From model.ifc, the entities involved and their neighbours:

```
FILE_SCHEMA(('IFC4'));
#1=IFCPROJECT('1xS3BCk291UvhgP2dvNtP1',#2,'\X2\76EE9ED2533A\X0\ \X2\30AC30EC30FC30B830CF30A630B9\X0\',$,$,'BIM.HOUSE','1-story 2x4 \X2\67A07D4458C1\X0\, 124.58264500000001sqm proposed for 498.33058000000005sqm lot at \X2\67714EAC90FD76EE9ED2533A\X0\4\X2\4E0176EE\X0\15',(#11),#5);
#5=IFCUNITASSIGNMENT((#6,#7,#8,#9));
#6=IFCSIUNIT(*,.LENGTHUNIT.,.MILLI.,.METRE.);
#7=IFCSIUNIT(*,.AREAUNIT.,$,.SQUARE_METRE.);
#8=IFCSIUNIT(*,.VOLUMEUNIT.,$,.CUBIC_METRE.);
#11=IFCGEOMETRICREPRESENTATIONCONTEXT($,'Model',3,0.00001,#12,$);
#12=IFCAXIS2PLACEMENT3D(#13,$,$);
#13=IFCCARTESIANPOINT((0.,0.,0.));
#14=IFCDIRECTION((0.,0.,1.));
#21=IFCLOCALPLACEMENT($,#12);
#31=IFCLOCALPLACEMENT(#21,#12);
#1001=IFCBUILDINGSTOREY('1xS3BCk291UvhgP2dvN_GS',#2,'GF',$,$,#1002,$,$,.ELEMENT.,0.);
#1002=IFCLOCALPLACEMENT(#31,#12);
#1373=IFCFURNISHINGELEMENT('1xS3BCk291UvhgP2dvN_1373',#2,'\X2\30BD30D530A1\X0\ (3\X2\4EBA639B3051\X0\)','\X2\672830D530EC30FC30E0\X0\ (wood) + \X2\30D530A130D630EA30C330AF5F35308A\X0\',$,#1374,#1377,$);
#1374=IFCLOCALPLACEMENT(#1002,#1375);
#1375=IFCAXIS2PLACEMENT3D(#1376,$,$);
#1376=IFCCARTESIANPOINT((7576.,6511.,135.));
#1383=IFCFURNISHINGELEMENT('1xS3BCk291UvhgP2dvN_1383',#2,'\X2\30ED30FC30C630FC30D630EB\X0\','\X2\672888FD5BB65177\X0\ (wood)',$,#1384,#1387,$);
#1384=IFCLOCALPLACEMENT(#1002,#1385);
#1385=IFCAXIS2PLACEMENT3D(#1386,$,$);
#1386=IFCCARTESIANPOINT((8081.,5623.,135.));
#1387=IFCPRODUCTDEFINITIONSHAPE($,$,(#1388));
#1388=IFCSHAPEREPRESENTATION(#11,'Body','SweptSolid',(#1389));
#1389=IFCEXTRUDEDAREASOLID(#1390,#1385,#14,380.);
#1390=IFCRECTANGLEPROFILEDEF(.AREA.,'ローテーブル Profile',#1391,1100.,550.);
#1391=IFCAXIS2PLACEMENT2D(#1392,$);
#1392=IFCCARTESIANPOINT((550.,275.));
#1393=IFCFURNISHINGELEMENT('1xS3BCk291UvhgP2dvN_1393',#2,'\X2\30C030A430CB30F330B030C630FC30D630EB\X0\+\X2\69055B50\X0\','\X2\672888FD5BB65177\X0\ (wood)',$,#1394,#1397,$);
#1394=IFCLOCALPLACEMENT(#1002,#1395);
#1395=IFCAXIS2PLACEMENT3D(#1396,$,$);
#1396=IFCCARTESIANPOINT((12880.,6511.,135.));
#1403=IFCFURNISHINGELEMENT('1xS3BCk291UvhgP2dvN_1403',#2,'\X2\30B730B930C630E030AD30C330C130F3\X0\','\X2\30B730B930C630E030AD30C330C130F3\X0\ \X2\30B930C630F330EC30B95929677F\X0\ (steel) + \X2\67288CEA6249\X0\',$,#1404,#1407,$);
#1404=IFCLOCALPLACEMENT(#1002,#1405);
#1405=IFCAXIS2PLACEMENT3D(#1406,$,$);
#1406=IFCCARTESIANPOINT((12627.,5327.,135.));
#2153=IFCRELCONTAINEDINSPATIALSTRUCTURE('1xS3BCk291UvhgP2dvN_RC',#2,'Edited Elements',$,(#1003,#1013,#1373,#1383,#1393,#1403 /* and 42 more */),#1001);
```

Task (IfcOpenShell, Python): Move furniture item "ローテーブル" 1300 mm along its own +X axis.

```python
import ifcopenshell
import ifcopenshell.api.geometry
import ifcopenshell.util.placement
import ifcopenshell.util.unit

model = ifcopenshell.open("model.ifc")
unit_scale = ifcopenshell.util.unit.calculate_unit_scale(model)

item = model.by_guid("1xS3BCk291UvhgP2dvN_1383")
matrix = ifcopenshell.util.placement.get_local_placement(item.ObjectPlacement)
matrix[:3, 3] += matrix[:3, 0] * 1.3 / unit_scale
ifcopenshell.api.geometry.edit_object_placement(model, product=item, matrix=matrix, is_si=False)

print(ifcopenshell.util.placement.get_local_placement(item.ObjectPlacement).round(3) + 0.0)

model.write("model_rev.ifc")
```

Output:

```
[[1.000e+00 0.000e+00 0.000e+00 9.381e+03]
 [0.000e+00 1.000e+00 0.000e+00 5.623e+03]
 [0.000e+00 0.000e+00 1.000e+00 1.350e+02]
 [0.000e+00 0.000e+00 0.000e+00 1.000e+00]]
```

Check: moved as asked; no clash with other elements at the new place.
